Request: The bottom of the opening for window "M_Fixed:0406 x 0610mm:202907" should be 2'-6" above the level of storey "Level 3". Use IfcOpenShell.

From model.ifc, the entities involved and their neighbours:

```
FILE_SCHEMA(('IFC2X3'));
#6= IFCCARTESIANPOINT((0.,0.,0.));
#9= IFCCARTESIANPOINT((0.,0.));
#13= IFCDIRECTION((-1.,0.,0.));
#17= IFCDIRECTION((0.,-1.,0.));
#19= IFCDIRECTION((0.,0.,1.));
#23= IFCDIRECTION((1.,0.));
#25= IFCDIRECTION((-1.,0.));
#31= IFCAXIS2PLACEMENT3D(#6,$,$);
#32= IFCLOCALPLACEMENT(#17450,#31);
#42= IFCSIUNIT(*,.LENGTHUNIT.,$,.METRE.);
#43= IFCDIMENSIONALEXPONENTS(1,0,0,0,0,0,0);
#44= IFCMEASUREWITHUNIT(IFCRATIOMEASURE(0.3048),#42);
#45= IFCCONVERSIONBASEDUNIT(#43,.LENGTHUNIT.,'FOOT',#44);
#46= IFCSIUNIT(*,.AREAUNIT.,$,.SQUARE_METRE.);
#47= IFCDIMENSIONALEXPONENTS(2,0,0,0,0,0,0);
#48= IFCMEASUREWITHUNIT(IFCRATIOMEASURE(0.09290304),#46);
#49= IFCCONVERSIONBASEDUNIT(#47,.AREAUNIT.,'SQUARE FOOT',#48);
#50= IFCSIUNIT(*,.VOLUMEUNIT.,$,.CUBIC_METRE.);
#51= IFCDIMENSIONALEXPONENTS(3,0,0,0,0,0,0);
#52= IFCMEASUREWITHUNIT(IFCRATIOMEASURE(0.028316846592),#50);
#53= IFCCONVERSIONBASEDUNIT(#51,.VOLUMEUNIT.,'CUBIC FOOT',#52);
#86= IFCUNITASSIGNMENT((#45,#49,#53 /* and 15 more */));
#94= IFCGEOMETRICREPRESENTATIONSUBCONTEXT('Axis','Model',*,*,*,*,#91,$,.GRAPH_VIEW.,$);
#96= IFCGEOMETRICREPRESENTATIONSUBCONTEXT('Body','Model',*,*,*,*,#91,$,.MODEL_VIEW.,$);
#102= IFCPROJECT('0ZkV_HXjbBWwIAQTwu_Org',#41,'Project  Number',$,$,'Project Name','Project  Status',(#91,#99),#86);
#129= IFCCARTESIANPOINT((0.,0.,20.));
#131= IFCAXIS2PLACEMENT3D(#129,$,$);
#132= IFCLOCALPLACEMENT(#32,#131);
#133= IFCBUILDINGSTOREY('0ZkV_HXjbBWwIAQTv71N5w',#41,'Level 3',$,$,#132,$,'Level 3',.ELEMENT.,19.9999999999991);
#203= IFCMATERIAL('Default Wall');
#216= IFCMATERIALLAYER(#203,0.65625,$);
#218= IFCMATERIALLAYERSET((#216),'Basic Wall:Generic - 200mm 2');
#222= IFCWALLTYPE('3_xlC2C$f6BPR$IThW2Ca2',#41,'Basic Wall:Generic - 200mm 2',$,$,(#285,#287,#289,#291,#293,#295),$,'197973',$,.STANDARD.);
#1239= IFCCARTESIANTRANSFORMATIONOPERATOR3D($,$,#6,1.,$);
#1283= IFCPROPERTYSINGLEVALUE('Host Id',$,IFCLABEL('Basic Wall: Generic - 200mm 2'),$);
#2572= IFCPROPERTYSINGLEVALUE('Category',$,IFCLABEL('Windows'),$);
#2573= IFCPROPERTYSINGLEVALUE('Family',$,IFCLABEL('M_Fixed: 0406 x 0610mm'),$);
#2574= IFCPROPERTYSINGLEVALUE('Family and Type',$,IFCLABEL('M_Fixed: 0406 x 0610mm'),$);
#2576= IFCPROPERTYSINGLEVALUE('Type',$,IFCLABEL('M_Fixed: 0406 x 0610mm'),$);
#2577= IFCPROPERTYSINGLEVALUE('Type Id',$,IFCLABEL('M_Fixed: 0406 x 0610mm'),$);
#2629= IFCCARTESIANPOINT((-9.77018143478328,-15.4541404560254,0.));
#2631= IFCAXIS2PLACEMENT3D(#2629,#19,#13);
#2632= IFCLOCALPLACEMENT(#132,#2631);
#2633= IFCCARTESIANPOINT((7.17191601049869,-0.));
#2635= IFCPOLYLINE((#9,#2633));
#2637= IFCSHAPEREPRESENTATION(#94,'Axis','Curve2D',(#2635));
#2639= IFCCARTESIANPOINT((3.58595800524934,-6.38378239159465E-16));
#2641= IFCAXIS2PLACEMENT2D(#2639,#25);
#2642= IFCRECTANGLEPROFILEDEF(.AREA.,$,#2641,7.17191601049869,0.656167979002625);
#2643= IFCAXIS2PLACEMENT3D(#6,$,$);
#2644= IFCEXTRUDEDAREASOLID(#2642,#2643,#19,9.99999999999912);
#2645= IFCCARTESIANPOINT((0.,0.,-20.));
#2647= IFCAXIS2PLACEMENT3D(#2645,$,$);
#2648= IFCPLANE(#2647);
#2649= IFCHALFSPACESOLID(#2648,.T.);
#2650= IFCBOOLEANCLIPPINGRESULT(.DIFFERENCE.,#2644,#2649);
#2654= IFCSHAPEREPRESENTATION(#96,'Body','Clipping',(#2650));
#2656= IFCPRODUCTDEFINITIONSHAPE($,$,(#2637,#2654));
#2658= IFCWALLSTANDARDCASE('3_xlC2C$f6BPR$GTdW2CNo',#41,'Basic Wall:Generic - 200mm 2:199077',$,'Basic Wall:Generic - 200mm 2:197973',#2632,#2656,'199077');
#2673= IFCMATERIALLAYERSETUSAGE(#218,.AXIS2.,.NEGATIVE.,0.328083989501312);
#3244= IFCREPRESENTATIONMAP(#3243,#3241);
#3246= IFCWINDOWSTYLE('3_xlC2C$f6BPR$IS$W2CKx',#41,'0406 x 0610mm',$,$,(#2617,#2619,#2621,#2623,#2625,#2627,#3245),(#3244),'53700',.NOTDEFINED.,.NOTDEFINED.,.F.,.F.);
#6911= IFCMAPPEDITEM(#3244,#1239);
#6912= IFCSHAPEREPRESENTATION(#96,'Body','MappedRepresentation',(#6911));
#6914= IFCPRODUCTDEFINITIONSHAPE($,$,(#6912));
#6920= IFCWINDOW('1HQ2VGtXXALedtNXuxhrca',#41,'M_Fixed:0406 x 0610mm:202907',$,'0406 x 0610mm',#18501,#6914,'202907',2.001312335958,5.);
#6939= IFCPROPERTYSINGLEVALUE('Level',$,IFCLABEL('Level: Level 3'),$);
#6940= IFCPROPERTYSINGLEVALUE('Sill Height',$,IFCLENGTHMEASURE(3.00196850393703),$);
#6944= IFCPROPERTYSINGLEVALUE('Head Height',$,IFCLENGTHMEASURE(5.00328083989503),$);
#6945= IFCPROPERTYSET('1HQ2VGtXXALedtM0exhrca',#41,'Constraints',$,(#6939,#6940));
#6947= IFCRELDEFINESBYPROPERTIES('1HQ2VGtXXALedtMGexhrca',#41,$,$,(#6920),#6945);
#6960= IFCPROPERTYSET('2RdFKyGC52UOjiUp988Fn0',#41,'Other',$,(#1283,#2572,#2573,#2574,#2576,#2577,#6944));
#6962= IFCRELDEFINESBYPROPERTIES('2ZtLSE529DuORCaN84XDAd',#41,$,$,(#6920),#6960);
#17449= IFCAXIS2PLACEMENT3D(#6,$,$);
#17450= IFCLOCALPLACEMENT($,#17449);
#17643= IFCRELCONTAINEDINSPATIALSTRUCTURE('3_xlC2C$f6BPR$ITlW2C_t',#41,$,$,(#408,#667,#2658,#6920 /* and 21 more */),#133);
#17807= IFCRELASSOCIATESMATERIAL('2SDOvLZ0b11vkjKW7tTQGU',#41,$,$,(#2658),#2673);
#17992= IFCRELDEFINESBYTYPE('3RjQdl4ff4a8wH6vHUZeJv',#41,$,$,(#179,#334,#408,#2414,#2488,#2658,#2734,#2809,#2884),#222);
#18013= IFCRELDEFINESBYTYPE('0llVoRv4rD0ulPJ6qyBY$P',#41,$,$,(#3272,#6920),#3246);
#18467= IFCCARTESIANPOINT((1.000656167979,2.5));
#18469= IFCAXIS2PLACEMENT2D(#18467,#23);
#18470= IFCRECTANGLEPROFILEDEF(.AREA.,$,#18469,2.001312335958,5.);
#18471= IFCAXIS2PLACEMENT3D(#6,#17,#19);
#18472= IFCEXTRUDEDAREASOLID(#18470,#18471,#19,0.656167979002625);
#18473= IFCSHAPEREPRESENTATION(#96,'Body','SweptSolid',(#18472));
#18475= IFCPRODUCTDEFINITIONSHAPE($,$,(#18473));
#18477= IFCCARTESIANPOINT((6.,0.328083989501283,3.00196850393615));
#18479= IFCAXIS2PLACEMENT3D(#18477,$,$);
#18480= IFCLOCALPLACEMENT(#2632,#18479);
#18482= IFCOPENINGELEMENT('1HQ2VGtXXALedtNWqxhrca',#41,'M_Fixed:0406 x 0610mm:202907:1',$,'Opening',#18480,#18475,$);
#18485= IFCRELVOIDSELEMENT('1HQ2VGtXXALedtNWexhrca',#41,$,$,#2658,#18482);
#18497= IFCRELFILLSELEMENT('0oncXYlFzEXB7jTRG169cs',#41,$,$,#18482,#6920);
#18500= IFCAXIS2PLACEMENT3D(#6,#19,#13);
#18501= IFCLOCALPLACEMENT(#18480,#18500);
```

```python
import numpy as np
import ifcopenshell
import ifcopenshell.api.geometry
import ifcopenshell.api.pset
import ifcopenshell.geom
import ifcopenshell.util.element
import ifcopenshell.util.placement
import ifcopenshell.util.shape
import ifcopenshell.util.unit

model = ifcopenshell.open("model.ifc")
unit_scale = ifcopenshell.util.unit.calculate_unit_scale(model)

window = model.by_guid("1HQ2VGtXXALedtNXuxhrca")
opening = window.FillsVoids[0].RelatingOpeningElement
storey = ifcopenshell.util.element.get_container(window, ifc_class="IfcBuildingStorey")
level = ifcopenshell.util.placement.get_local_placement(storey.ObjectPlacement)[2, 3]

# The opening's origin need not be at the sill, so measure its lowest point.
shape = ifcopenshell.geom.create_shape(ifcopenshell.geom.settings(), opening)
bottom = ifcopenshell.util.shape.get_shape_bottom_elevation(shape, shape.geometry) / unit_scale
dz = level + 30 * 0.0254 / unit_scale - bottom

shift = np.array([0.0, 0.0, dz])
# The window is placed relative to its opening, so it follows when the opening moves.
matrix = ifcopenshell.util.placement.get_local_placement(opening.ObjectPlacement)
matrix[:3, 3] += shift
ifcopenshell.api.geometry.edit_object_placement(
    model, product=opening, matrix=matrix, is_si=False, should_transform_children=True
)

# Keep the stored heights in step.
pset = model.by_id(ifcopenshell.util.element.get_pset(window, "Constraints", should_inherit=False)["id"])
ifcopenshell.api.pset.edit_pset(model, pset=pset, properties={
    "Sill Height": model.create_entity("IfcLengthMeasure", ifcopenshell.util.element.get_pset(window, "Constraints", "Sill Height") + dz),
})
pset = model.by_id(ifcopenshell.util.element.get_pset(window, "Other", should_inherit=False)["id"])
ifcopenshell.api.pset.edit_pset(model, pset=pset, properties={
    "Head Height": model.create_entity("IfcLengthMeasure", ifcopenshell.util.element.get_pset(window, "Other", "Head Height") + dz),
})

print(f"moved by {dz * unit_scale:+.3f} m")

model.write("model_updated.ifc")
```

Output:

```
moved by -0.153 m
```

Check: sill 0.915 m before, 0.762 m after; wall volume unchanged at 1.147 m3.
